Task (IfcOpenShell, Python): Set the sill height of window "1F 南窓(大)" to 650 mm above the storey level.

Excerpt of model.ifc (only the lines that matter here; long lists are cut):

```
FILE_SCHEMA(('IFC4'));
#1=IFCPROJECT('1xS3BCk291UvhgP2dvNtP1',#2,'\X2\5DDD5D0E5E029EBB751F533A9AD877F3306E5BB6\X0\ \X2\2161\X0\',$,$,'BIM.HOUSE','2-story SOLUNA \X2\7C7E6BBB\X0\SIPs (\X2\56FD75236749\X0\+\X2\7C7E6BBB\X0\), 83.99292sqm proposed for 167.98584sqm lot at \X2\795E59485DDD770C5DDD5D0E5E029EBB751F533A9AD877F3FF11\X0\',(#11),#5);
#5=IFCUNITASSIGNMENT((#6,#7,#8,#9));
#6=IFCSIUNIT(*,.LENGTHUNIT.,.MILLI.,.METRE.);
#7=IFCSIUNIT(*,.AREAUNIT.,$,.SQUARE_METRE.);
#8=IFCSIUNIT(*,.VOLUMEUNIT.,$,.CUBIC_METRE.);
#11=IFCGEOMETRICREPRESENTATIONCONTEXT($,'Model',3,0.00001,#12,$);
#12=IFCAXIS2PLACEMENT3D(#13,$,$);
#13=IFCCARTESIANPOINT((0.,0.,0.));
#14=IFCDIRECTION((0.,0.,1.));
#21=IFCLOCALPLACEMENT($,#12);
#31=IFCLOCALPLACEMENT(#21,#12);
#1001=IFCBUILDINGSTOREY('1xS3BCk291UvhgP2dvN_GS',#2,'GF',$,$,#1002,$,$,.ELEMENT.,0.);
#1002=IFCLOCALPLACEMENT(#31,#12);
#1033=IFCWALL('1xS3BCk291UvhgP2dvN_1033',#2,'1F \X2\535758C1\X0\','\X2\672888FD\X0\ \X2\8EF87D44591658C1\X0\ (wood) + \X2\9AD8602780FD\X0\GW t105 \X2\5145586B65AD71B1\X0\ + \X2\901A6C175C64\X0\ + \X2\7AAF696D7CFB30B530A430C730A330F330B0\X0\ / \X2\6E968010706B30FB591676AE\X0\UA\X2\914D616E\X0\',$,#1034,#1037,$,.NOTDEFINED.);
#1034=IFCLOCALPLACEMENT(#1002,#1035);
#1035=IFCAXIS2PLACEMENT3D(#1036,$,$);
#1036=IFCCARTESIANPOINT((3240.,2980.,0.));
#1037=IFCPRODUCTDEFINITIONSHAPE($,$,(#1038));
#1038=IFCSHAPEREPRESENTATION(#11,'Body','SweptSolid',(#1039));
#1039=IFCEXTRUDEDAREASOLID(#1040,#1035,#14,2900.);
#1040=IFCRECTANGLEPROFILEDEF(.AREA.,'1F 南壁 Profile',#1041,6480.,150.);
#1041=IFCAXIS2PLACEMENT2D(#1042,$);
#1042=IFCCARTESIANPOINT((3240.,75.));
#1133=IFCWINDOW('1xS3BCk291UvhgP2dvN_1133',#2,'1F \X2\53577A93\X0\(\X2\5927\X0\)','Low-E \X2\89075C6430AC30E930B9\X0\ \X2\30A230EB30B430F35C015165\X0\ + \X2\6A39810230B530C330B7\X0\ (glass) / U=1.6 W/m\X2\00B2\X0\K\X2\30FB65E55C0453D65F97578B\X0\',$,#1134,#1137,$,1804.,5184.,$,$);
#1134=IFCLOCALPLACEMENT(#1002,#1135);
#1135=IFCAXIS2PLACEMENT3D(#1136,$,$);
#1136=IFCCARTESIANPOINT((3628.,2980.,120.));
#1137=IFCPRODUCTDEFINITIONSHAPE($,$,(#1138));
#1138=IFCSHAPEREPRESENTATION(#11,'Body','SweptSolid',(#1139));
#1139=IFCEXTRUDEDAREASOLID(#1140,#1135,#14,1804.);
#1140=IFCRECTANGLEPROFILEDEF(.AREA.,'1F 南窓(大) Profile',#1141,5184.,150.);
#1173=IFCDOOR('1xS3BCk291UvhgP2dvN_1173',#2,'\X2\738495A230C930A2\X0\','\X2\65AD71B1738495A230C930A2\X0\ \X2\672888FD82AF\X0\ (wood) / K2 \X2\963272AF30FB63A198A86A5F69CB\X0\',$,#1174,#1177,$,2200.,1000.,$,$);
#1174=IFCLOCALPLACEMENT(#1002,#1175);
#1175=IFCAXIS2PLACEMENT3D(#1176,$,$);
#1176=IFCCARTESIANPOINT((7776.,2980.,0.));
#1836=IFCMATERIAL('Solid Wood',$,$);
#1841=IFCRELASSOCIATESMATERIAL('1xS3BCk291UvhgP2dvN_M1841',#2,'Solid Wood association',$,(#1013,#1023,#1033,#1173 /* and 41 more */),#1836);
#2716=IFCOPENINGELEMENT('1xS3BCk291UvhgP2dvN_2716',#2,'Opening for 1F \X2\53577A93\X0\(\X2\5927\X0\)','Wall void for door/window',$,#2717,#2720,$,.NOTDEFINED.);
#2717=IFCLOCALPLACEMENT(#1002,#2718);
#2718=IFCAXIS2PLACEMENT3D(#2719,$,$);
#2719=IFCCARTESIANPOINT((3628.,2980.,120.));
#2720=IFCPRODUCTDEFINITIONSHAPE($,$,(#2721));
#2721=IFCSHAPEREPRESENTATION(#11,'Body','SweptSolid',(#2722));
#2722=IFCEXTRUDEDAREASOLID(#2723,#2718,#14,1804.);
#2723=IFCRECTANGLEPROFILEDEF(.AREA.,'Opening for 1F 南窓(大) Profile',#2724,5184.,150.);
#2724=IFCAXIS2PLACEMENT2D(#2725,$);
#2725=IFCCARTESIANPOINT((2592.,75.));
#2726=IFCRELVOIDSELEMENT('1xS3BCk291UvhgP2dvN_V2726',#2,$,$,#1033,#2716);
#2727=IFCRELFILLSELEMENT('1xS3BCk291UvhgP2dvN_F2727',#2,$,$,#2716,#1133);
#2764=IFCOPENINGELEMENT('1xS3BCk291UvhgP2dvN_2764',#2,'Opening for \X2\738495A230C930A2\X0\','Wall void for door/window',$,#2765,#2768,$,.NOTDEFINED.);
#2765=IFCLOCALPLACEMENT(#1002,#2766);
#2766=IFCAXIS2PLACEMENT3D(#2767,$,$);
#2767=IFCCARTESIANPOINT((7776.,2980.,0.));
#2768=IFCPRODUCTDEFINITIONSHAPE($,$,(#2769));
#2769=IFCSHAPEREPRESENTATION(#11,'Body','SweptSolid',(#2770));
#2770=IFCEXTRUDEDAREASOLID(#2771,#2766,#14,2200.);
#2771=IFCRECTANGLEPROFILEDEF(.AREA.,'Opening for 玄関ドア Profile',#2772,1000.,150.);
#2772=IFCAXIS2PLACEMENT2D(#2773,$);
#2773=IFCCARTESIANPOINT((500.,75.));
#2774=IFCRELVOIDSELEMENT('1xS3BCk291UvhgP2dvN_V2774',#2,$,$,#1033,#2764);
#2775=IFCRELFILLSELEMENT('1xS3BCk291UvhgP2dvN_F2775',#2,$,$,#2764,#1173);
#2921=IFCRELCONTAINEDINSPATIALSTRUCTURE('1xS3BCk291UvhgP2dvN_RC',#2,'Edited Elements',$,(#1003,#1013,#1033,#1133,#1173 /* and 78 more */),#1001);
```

```python
import numpy as np
import ifcopenshell
import ifcopenshell.api.geometry
import ifcopenshell.geom
import ifcopenshell.util.element
import ifcopenshell.util.placement
import ifcopenshell.util.shape
import ifcopenshell.util.unit

model = ifcopenshell.open("model.ifc")
unit_scale = ifcopenshell.util.unit.calculate_unit_scale(model)

window = model.by_guid("1xS3BCk291UvhgP2dvN_1133")
opening = window.FillsVoids[0].RelatingOpeningElement
storey = ifcopenshell.util.element.get_container(window, ifc_class="IfcBuildingStorey")
level = ifcopenshell.util.placement.get_local_placement(storey.ObjectPlacement)[2, 3]

# The opening's origin need not be at the sill, so measure its lowest point.
shape = ifcopenshell.geom.create_shape(ifcopenshell.geom.settings(), opening)
bottom = ifcopenshell.util.shape.get_shape_bottom_elevation(shape, shape.geometry) / unit_scale
dz = level + 0.65 / unit_scale - bottom

shift = np.array([0.0, 0.0, dz])
# The window is not placed relative to its opening, so move both.
for product in (opening, window):
    matrix = ifcopenshell.util.placement.get_local_placement(product.ObjectPlacement)
    matrix[:3, 3] += shift
    ifcopenshell.api.geometry.edit_object_placement(model, product=product, matrix=matrix, is_si=False)

print(f"moved by {dz * unit_scale:+.3f} m")

model.write("model_rev.ifc")
```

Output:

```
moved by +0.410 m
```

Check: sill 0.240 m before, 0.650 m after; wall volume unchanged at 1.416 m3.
